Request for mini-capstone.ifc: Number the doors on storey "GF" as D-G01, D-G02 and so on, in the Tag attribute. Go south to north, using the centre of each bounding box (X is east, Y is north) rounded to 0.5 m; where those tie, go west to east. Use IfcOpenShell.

First a look at what the model holds.

```python
import ifcopenshell
import ifcopenshell.util.element
import ifcopenshell.util.placement

model = ifcopenshell.open("mini-capstone.ifc")
print(model.schema)
storey = next(s for s in model.by_type("IfcBuildingStorey") if s.Name == "GF")
doors = [e for e in ifcopenshell.util.element.get_decomposition(storey) if e.is_a("IfcDoor")]
for e in sorted(doors, key=lambda e: e.id()):
    origin = ifcopenshell.util.placement.get_local_placement(e.ObjectPlacement)[:3, 3]
    print(e.id(), e.Tag, e.Name, origin.round(2) + 0.0, sep=" | ")
```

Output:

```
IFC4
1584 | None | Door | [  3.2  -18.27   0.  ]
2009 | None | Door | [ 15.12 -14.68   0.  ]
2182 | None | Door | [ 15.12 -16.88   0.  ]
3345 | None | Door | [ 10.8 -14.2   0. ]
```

```python
import ifcopenshell
import ifcopenshell.geom
import ifcopenshell.util.element
import ifcopenshell.util.shape

model = ifcopenshell.open("mini-capstone.ifc")
settings = ifcopenshell.geom.settings()
settings.set("use-world-coords", True)


def centre(element):
    shape = ifcopenshell.geom.create_shape(settings, element)
    return ifcopenshell.util.shape.get_bbox_centroid(shape.geometry)


storey = next(s for s in model.by_type("IfcBuildingStorey") if s.Name == "GF")
doors = [e for e in ifcopenshell.util.element.get_decomposition(storey) if e.is_a("IfcDoor")]

# Insertion points can sit at a corner or the storey origin, so sort by the geometry (in metres).
centres = {e: centre(e) for e in doors}
doors.sort(key=lambda e: (round(centres[e][1] / 0.5), centres[e][0]))

for i, e in enumerate(doors, start=1):
    number = f"D-G{i:02d}"
    e.Tag = number
    print(e.id(), number)

model.write("mini-capstone-out.ifc")
```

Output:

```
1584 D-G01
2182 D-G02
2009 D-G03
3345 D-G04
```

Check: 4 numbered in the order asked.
